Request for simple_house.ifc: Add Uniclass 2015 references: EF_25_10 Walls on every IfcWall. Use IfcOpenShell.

First a look at what the model holds.

```python
import ifcopenshell

model = ifcopenshell.open("simple_house.ifc")
print(model.schema)
print("classifications:", [c.Name for c in model.by_type("IfcClassification")])
for ifc_class in ("IfcDoor", "IfcRoof", "IfcStair", "IfcWall", "IfcWindow"):
    print(ifc_class, len(model.by_type(ifc_class)))
```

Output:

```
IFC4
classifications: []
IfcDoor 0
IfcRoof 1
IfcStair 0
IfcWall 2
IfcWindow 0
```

```python
import ifcopenshell
import ifcopenshell.api.classification

model = ifcopenshell.open("simple_house.ifc")

system = ifcopenshell.api.classification.add_classification(model, classification="Uniclass 2015")

codes = {
    "IfcWall": ("EF_25_10", "Walls"),
}
for ifc_class, (code, name) in codes.items():
    products = model.by_type(ifc_class)
    ifcopenshell.api.classification.add_reference(
        model, products=products, classification=system, identification=code, name=name
    )
    print(code, len(products))

model.write("simple_house_rev.ifc")
```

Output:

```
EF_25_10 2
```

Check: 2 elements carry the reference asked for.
